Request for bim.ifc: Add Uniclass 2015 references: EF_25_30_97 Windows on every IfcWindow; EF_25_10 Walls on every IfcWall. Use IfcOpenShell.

First a look at what the model holds.

```python
import ifcopenshell

model = ifcopenshell.open("bim.ifc")
print(model.schema)
print("classifications:", [c.Name for c in model.by_type("IfcClassification")])
for ifc_class in ("IfcDoor", "IfcRoof", "IfcStair", "IfcWall", "IfcWindow"):
    print(ifc_class, len(model.by_type(ifc_class)))
```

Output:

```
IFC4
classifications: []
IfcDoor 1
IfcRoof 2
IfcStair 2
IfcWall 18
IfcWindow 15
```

```python
import ifcopenshell
import ifcopenshell.api.classification

model = ifcopenshell.open("bim.ifc")

system = ifcopenshell.api.classification.add_classification(model, classification="Uniclass 2015")

codes = {
    "IfcWindow": ("EF_25_30_97", "Windows"),
    "IfcWall": ("EF_25_10", "Walls"),
}
for ifc_class, (code, name) in codes.items():
    products = model.by_type(ifc_class)
    ifcopenshell.api.classification.add_reference(
        model, products=products, classification=system, identification=code, name=name
    )
    print(code, len(products))

model.write("bim_v2.ifc")
```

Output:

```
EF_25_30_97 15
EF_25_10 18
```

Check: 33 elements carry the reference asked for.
